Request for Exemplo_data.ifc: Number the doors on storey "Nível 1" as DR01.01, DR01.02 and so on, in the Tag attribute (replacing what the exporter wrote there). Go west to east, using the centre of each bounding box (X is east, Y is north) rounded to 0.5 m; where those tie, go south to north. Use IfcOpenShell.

First a look at what the model holds.

```python
import ifcopenshell
import ifcopenshell.util.element
import ifcopenshell.util.placement

model = ifcopenshell.open("Exemplo_data.ifc")
print(model.schema)
storey = next(s for s in model.by_type("IfcBuildingStorey") if s.Name == "Nível 1")
doors = [e for e in ifcopenshell.util.element.get_decomposition(storey) if e.is_a("IfcDoor")]
for e in sorted(doors, key=lambda e: e.id()):
    origin = ifcopenshell.util.placement.get_local_placement(e.ObjectPlacement)[:3, 3]
    print(e.id(), e.Tag, e.Name, origin.round(2) + 0.0, sep=" | ")
```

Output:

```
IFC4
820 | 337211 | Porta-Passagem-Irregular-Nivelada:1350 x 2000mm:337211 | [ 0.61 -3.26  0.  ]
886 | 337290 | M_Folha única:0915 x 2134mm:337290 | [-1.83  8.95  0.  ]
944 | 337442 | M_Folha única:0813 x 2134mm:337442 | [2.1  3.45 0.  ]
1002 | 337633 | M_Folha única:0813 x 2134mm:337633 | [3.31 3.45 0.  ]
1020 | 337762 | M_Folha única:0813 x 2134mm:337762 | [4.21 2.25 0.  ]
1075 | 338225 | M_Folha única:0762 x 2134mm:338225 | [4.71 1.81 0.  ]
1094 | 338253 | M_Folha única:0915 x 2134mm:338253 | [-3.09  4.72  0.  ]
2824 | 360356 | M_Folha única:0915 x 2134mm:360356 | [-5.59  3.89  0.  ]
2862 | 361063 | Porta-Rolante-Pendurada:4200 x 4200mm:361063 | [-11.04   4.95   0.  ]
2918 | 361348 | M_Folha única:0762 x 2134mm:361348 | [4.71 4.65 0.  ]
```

```python
import ifcopenshell
import ifcopenshell.geom
import ifcopenshell.util.element
import ifcopenshell.util.shape

model = ifcopenshell.open("Exemplo_data.ifc")
settings = ifcopenshell.geom.settings()
settings.set("use-world-coords", True)


def centre(element):
    shape = ifcopenshell.geom.create_shape(settings, element)
    return ifcopenshell.util.shape.get_bbox_centroid(shape.geometry)


storey = next(s for s in model.by_type("IfcBuildingStorey") if s.Name == "Nível 1")
doors = [e for e in ifcopenshell.util.element.get_decomposition(storey) if e.is_a("IfcDoor")]

# Insertion points can sit at a corner or the storey origin, so sort by the geometry (in metres).
centres = {e: centre(e) for e in doors}
doors.sort(key=lambda e: (round(centres[e][0] / 0.5), centres[e][1]))

for i, e in enumerate(doors, start=1):
    number = f"DR01.{i:02d}"
    e.Tag = number
    print(e.id(), number)

model.write("Exemplo_data_edited.ifc")
```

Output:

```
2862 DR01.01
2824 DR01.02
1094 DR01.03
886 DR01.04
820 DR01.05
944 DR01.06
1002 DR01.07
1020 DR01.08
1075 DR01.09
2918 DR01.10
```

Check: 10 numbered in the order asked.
